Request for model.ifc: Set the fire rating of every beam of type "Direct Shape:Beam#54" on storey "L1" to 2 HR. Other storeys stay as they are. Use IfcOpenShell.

First a look at what the model holds.

```python
import ifcopenshell
import ifcopenshell.util.element

model = ifcopenshell.open("model.ifc")
print(model.schema)
storey = next(s for s in model.by_type("IfcBuildingStorey") if s.Name == "L1")
beams = [e for e in ifcopenshell.util.element.get_decomposition(storey) if e.is_a("IfcBeam")]
seen = {}
for e in beams:
    element_type = ifcopenshell.util.element.get_type(e)
    key = (element_type.Name if element_type != e and element_type else None, ifcopenshell.util.element.get_pset(e, "Pset_BeamCommon", "FireRating"))
    seen[key] = seen.get(key, 0) + 1
for (name, value), count in sorted(seen.items(), key=str):
    print(count, "x", name, "|", value)
```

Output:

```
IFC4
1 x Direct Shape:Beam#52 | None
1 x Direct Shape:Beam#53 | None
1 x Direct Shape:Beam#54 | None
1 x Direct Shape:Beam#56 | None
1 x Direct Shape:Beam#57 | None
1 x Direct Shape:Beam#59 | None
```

```python
import ifcopenshell
import ifcopenshell.api.pset
import ifcopenshell.util.element

model = ifcopenshell.open("model.ifc")

storey = next(s for s in model.by_type("IfcBuildingStorey") if s.Name == "L1")
beams = [e for e in ifcopenshell.util.element.get_decomposition(storey) if e.is_a("IfcBeam")]

count = 0
for e in beams:
    element_type = ifcopenshell.util.element.get_type(e)
    if element_type in (None, e) or element_type.Name != "Direct Shape:Beam#54":
        continue
    # add_pset returns the element's existing set when there is one.
    pset = ifcopenshell.api.pset.add_pset(model, product=e, name="Pset_BeamCommon")
    ifcopenshell.api.pset.edit_pset(model, pset=pset, properties={"FireRating": "2 HR"})
    count += 1

print(count, "beams updated")

model.write("model-out.ifc")
```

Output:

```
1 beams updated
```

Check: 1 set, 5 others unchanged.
